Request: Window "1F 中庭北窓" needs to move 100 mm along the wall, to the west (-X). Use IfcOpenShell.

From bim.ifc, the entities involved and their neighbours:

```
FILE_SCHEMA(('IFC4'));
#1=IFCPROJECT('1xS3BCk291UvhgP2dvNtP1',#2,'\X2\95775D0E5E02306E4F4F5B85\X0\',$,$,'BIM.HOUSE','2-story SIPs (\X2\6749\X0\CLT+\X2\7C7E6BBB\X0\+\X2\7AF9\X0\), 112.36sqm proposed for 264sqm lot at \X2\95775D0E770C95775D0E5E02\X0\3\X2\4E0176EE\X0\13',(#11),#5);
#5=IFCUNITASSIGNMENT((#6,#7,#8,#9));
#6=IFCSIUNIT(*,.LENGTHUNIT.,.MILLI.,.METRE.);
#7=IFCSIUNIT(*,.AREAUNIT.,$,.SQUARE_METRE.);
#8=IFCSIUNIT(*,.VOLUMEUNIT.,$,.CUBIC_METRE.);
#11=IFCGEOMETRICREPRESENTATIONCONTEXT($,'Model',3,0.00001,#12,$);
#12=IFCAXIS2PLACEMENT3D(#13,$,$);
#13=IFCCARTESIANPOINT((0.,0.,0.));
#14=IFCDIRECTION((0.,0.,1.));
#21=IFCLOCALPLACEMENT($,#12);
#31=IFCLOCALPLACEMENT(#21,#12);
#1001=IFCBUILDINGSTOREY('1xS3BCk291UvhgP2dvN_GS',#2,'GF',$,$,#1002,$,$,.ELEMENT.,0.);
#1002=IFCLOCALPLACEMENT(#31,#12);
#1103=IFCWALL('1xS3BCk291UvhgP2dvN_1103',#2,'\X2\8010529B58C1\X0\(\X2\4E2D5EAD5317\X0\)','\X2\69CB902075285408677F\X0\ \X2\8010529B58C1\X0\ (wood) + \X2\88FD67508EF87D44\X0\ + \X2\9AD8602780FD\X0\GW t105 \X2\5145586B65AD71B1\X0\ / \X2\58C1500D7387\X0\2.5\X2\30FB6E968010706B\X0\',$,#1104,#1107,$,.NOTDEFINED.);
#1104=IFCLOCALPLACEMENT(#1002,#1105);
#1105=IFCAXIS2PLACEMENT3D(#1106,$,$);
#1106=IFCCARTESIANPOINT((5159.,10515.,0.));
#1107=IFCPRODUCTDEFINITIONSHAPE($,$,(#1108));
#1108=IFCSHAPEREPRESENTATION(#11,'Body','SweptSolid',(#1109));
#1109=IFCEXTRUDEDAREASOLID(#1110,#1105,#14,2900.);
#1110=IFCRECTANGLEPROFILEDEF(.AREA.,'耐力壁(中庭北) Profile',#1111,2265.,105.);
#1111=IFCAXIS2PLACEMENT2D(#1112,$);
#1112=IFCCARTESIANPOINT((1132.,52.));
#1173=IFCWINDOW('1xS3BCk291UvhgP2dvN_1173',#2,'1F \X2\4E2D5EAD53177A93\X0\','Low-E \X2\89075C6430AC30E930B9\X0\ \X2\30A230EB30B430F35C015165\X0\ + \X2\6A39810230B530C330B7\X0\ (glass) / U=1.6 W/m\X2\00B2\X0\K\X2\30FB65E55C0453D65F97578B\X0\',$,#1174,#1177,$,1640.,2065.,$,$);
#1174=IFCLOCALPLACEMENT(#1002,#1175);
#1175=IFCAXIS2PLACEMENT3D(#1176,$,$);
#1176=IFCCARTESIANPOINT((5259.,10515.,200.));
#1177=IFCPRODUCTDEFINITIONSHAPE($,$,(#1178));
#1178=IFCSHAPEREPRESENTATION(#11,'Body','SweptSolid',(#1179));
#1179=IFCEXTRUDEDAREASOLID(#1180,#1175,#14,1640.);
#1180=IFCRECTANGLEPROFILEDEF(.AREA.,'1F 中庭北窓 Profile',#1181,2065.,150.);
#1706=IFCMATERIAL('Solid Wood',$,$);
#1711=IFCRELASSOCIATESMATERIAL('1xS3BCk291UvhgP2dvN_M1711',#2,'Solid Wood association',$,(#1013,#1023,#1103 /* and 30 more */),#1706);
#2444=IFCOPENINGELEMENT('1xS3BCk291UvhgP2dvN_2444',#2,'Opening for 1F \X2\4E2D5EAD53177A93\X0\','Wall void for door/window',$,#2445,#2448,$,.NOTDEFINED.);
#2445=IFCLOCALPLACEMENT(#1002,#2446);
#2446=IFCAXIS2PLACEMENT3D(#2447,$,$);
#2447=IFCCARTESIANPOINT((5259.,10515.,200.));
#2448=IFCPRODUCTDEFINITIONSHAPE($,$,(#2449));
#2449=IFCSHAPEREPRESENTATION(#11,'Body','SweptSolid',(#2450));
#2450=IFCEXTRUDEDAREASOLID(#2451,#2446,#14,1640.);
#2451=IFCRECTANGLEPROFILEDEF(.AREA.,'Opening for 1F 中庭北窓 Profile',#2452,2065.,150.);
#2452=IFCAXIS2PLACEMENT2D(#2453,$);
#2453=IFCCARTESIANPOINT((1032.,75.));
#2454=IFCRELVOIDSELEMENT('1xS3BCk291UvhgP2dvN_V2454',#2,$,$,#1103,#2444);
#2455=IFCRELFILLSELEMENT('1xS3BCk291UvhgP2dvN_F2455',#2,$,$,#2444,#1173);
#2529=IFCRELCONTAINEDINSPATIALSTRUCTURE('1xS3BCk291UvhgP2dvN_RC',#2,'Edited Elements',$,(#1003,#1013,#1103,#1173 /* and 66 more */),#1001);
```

```python
import ifcopenshell
import ifcopenshell.api.geometry
import ifcopenshell.util.placement
import ifcopenshell.util.unit

model = ifcopenshell.open("bim.ifc")
unit_scale = ifcopenshell.util.unit.calculate_unit_scale(model)

window = model.by_guid("1xS3BCk291UvhgP2dvN_1173")
opening = window.FillsVoids[0].RelatingOpeningElement
wall = opening.VoidsElements[0].RelatingBuildingElement

wall_matrix = ifcopenshell.util.placement.get_local_placement(wall.ObjectPlacement)
shift = wall_matrix[:3, 0] * -0.1 / unit_scale
before = ifcopenshell.util.placement.get_local_placement(window.ObjectPlacement)[:3, 3].copy()

# The window is not placed relative to its opening, so move both.
for product in (opening, window):
    matrix = ifcopenshell.util.placement.get_local_placement(product.ObjectPlacement)
    matrix[:3, 3] += shift
    ifcopenshell.api.geometry.edit_object_placement(model, product=product, matrix=matrix, is_si=False)

after = ifcopenshell.util.placement.get_local_placement(window.ObjectPlacement)[:3, 3]
print("window moved by", (after - before).round(3) + 0.0)

model.write("bim_rev.ifc")
```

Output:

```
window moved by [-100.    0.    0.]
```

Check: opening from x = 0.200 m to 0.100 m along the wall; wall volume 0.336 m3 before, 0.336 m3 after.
